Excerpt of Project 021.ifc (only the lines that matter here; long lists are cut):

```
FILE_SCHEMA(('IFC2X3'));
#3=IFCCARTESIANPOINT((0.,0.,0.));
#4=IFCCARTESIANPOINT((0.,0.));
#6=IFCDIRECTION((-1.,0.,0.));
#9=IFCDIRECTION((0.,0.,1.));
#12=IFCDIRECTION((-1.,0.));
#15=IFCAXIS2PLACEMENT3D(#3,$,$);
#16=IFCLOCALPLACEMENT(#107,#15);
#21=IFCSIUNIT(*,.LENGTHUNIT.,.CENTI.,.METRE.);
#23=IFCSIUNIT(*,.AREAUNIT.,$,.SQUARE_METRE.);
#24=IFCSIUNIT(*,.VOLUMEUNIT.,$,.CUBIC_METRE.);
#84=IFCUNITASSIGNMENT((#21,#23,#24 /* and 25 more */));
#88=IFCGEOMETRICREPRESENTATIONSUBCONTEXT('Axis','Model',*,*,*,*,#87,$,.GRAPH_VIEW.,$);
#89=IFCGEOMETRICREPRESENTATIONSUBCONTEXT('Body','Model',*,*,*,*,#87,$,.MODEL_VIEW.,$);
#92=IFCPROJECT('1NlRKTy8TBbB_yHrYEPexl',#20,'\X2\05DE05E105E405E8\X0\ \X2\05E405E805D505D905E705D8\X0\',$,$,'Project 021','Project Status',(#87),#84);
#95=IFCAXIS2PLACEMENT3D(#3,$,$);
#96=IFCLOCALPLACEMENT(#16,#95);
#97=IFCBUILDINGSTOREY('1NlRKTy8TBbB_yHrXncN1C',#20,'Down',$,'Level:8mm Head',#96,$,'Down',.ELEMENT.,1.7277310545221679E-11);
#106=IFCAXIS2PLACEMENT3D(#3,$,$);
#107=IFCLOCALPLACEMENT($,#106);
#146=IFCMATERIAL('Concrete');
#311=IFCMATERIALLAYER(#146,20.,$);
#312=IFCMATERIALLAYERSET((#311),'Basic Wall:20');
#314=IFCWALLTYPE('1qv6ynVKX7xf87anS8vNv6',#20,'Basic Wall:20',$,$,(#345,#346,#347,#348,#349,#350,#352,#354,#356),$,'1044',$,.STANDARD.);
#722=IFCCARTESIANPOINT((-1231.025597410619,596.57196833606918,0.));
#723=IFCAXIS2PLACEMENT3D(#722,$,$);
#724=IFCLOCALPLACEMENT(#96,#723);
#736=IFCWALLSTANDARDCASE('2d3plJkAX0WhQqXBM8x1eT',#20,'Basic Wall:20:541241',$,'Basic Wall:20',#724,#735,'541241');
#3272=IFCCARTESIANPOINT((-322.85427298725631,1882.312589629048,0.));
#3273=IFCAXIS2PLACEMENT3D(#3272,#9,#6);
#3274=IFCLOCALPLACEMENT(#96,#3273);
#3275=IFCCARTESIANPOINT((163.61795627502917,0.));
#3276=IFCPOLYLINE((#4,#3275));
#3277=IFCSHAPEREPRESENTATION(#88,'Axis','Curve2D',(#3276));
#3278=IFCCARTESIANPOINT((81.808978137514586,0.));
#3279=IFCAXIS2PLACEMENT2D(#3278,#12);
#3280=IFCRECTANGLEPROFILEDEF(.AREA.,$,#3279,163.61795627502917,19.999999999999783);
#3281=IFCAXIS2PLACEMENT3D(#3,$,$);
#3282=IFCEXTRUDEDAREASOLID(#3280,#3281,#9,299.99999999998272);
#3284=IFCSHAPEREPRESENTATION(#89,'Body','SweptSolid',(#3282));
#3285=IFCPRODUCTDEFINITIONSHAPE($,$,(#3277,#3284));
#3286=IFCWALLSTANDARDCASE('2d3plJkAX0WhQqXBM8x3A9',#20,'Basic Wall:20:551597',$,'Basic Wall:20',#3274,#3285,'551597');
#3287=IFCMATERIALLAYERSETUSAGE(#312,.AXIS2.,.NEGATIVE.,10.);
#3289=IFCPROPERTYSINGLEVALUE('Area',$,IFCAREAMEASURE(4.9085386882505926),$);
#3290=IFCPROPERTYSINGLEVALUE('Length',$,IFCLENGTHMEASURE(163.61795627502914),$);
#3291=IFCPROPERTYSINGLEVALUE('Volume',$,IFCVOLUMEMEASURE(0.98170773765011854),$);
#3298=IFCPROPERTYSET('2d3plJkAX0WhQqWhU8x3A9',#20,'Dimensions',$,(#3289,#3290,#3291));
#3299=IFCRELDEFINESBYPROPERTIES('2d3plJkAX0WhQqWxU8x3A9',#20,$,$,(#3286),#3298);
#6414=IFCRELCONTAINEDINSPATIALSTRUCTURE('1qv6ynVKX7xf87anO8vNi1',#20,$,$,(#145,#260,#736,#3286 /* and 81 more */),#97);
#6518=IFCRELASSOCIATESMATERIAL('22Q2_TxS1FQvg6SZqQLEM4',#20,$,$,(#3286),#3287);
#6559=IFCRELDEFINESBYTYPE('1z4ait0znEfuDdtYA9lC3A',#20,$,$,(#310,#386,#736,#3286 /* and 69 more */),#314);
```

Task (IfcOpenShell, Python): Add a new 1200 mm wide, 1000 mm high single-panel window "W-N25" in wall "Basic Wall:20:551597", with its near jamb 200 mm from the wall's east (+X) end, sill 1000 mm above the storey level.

```python
import numpy as np
import ifcopenshell
import ifcopenshell.api.feature
import ifcopenshell.api.geometry
import ifcopenshell.api.pset
import ifcopenshell.api.root
import ifcopenshell.api.spatial
import ifcopenshell.api.type
import ifcopenshell.geom
import ifcopenshell.util.element
import ifcopenshell.util.placement
import ifcopenshell.util.representation
import ifcopenshell.util.shape
import ifcopenshell.util.unit

model = ifcopenshell.open("Project 021.ifc")
unit_scale = ifcopenshell.util.unit.calculate_unit_scale(model)
area_scale = ifcopenshell.util.unit.calculate_unit_scale(model, "AREAUNIT")
volume_scale = ifcopenshell.util.unit.calculate_unit_scale(model, "VOLUMEUNIT")
settings = ifcopenshell.geom.settings()


def volume(element):
    """Net volume in cubic metres, openings subtracted."""
    shape = ifcopenshell.geom.create_shape(settings, element)
    return ifcopenshell.util.shape.get_volume(shape.geometry)


wall = model.by_id(3286)
storey = ifcopenshell.util.element.get_container(wall, ifc_class="IfcBuildingStorey")
context = ifcopenshell.util.representation.get_context(model, "Model", "Body", "MODEL_VIEW")
before = volume(wall)

width, height, from_end, sill = 1.2, 1, 0.2, 1  # metres

# The wall runs along its own X axis, and the end named is its -X end.
wall_shape = ifcopenshell.geom.create_shape(settings, wall)
x, y, z = ifcopenshell.util.shape.get_vertices(wall_shape.geometry).T
start = x.min() + from_end
face, thickness = float(y.min()), float(y.max() - y.min())
wall_matrix = ifcopenshell.util.placement.get_local_placement(wall.ObjectPlacement)
level = ifcopenshell.util.placement.get_local_placement(storey.ObjectPlacement)[2, 3]


def in_wall(x, y):
    """Placement at x, y metres in the wall's axes, at sill height."""
    matrix = wall_matrix.copy()
    matrix[:, 3] = wall_matrix @ np.array([x / unit_scale, y / unit_scale, 0.0, 1.0])
    matrix[2, 3] = level + sill / unit_scale
    return matrix


# Opening: a box that overshoots both wall faces by 50 mm.
opening = ifcopenshell.api.root.create_entity(model, ifc_class="IfcOpeningElement")
box = ifcopenshell.api.geometry.add_wall_representation(
    model, context=context, length=width, height=height, thickness=thickness + 0.1
)
ifcopenshell.api.geometry.assign_representation(model, product=opening, representation=box)
ifcopenshell.api.geometry.edit_object_placement(model, product=opening, matrix=in_wall(start, face - 0.05), is_si=False)
ifcopenshell.api.feature.add_feature(model, feature=opening, element=wall)

window = ifcopenshell.api.root.create_entity(model, ifc_class="IfcWindow", name="W-N25")
window.OverallWidth, window.OverallHeight = width / unit_scale, height / unit_scale
body = ifcopenshell.api.geometry.add_window_representation(
    model,
    context=context,
    overall_width=window.OverallWidth,
    overall_height=window.OverallHeight,
    partition_type="SINGLE_PANEL",
)
ifcopenshell.api.geometry.assign_representation(model, product=window, representation=body)
ifcopenshell.api.spatial.assign_container(model, products=[window], relating_structure=storey)
fills = ifcopenshell.api.feature.add_filling(model, opening=opening, element=window)
fills.OwnerHistory = window.OwnerHistory  # required in IFC2X3

# IFC2X3 keeps the operation on the window style.
style = ifcopenshell.api.root.create_entity(model, ifc_class="IfcWindowStyle", name="W-N25")
style.OperationType, style.ConstructionType = "SINGLE_PANEL", "NOTDEFINED"
style.ParameterTakesPrecedence = style.Sizeable = False
ifcopenshell.api.type.assign_type(model, related_objects=[window], relating_type=style)

# Centre the window in the wall's thickness.
ifcopenshell.api.geometry.edit_object_placement(model, product=window, matrix=in_wall(start, face), is_si=False)
window_shape = ifcopenshell.geom.create_shape(settings, window)
depth = ifcopenshell.util.shape.get_vertices(window_shape.geometry)[:, 1]
offset = face + thickness / 2 - (depth.min() + depth.max()) / 2
ifcopenshell.api.geometry.edit_object_placement(model, product=window, matrix=in_wall(start, offset), is_si=False)

after = volume(wall)

# Update the wall's stored quantities.
pset = model.by_id(ifcopenshell.util.element.get_pset(wall, "Dimensions", should_inherit=False)["id"])
ifcopenshell.api.pset.edit_pset(model, pset=pset, properties={
    "Area": model.create_entity("IfcAreaMeasure", after / thickness / area_scale),
    "Volume": model.create_entity("IfcVolumeMeasure", after / volume_scale),
})

print(f"wall volume {before:.3f} -> {after:.3f} m3")

model.write("Project 021_v2.ifc")
```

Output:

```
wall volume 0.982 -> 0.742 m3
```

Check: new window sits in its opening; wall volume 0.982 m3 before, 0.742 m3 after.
